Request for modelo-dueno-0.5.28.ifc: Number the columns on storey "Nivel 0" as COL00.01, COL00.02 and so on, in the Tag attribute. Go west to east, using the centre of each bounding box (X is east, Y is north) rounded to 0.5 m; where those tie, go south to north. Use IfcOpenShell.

First a look at what the model holds.

```python
import ifcopenshell
import ifcopenshell.util.element
import ifcopenshell.util.placement

model = ifcopenshell.open("modelo-dueno-0.5.28.ifc")
print(model.schema)
storey = next(s for s in model.by_type("IfcBuildingStorey") if s.Name == "Nivel 0")
columns = [e for e in ifcopenshell.util.element.get_decomposition(storey) if e.is_a("IfcColumn")]
for e in sorted(columns, key=lambda e: e.id()):
    origin = ifcopenshell.util.placement.get_local_placement(e.ObjectPlacement)[:3, 3]
    print(e.id(), e.Tag, e.Name, origin.round(2) + 0.0, sep=" | ")
```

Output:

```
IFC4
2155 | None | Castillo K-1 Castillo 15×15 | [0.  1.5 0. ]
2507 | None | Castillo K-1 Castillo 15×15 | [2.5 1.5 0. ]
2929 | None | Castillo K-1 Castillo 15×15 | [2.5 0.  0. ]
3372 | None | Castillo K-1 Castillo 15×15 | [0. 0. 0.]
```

```python
import ifcopenshell
import ifcopenshell.geom
import ifcopenshell.util.element
import ifcopenshell.util.shape

model = ifcopenshell.open("modelo-dueno-0.5.28.ifc")
settings = ifcopenshell.geom.settings()
settings.set("use-world-coords", True)


def centre(element):
    shape = ifcopenshell.geom.create_shape(settings, element)
    return ifcopenshell.util.shape.get_bbox_centroid(shape.geometry)


storey = next(s for s in model.by_type("IfcBuildingStorey") if s.Name == "Nivel 0")
columns = [e for e in ifcopenshell.util.element.get_decomposition(storey) if e.is_a("IfcColumn")]

# Insertion points can sit at a corner or the storey origin, so sort by the geometry (in metres).
centres = {e: centre(e) for e in columns}
columns.sort(key=lambda e: (round(centres[e][0] / 0.5), centres[e][1]))

for i, e in enumerate(columns, start=1):
    number = f"COL00.{i:02d}"
    e.Tag = number
    print(e.id(), number)

model.write("modelo-dueno-0.5.28_rev.ifc")
```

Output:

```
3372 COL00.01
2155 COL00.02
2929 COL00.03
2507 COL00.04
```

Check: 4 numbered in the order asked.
